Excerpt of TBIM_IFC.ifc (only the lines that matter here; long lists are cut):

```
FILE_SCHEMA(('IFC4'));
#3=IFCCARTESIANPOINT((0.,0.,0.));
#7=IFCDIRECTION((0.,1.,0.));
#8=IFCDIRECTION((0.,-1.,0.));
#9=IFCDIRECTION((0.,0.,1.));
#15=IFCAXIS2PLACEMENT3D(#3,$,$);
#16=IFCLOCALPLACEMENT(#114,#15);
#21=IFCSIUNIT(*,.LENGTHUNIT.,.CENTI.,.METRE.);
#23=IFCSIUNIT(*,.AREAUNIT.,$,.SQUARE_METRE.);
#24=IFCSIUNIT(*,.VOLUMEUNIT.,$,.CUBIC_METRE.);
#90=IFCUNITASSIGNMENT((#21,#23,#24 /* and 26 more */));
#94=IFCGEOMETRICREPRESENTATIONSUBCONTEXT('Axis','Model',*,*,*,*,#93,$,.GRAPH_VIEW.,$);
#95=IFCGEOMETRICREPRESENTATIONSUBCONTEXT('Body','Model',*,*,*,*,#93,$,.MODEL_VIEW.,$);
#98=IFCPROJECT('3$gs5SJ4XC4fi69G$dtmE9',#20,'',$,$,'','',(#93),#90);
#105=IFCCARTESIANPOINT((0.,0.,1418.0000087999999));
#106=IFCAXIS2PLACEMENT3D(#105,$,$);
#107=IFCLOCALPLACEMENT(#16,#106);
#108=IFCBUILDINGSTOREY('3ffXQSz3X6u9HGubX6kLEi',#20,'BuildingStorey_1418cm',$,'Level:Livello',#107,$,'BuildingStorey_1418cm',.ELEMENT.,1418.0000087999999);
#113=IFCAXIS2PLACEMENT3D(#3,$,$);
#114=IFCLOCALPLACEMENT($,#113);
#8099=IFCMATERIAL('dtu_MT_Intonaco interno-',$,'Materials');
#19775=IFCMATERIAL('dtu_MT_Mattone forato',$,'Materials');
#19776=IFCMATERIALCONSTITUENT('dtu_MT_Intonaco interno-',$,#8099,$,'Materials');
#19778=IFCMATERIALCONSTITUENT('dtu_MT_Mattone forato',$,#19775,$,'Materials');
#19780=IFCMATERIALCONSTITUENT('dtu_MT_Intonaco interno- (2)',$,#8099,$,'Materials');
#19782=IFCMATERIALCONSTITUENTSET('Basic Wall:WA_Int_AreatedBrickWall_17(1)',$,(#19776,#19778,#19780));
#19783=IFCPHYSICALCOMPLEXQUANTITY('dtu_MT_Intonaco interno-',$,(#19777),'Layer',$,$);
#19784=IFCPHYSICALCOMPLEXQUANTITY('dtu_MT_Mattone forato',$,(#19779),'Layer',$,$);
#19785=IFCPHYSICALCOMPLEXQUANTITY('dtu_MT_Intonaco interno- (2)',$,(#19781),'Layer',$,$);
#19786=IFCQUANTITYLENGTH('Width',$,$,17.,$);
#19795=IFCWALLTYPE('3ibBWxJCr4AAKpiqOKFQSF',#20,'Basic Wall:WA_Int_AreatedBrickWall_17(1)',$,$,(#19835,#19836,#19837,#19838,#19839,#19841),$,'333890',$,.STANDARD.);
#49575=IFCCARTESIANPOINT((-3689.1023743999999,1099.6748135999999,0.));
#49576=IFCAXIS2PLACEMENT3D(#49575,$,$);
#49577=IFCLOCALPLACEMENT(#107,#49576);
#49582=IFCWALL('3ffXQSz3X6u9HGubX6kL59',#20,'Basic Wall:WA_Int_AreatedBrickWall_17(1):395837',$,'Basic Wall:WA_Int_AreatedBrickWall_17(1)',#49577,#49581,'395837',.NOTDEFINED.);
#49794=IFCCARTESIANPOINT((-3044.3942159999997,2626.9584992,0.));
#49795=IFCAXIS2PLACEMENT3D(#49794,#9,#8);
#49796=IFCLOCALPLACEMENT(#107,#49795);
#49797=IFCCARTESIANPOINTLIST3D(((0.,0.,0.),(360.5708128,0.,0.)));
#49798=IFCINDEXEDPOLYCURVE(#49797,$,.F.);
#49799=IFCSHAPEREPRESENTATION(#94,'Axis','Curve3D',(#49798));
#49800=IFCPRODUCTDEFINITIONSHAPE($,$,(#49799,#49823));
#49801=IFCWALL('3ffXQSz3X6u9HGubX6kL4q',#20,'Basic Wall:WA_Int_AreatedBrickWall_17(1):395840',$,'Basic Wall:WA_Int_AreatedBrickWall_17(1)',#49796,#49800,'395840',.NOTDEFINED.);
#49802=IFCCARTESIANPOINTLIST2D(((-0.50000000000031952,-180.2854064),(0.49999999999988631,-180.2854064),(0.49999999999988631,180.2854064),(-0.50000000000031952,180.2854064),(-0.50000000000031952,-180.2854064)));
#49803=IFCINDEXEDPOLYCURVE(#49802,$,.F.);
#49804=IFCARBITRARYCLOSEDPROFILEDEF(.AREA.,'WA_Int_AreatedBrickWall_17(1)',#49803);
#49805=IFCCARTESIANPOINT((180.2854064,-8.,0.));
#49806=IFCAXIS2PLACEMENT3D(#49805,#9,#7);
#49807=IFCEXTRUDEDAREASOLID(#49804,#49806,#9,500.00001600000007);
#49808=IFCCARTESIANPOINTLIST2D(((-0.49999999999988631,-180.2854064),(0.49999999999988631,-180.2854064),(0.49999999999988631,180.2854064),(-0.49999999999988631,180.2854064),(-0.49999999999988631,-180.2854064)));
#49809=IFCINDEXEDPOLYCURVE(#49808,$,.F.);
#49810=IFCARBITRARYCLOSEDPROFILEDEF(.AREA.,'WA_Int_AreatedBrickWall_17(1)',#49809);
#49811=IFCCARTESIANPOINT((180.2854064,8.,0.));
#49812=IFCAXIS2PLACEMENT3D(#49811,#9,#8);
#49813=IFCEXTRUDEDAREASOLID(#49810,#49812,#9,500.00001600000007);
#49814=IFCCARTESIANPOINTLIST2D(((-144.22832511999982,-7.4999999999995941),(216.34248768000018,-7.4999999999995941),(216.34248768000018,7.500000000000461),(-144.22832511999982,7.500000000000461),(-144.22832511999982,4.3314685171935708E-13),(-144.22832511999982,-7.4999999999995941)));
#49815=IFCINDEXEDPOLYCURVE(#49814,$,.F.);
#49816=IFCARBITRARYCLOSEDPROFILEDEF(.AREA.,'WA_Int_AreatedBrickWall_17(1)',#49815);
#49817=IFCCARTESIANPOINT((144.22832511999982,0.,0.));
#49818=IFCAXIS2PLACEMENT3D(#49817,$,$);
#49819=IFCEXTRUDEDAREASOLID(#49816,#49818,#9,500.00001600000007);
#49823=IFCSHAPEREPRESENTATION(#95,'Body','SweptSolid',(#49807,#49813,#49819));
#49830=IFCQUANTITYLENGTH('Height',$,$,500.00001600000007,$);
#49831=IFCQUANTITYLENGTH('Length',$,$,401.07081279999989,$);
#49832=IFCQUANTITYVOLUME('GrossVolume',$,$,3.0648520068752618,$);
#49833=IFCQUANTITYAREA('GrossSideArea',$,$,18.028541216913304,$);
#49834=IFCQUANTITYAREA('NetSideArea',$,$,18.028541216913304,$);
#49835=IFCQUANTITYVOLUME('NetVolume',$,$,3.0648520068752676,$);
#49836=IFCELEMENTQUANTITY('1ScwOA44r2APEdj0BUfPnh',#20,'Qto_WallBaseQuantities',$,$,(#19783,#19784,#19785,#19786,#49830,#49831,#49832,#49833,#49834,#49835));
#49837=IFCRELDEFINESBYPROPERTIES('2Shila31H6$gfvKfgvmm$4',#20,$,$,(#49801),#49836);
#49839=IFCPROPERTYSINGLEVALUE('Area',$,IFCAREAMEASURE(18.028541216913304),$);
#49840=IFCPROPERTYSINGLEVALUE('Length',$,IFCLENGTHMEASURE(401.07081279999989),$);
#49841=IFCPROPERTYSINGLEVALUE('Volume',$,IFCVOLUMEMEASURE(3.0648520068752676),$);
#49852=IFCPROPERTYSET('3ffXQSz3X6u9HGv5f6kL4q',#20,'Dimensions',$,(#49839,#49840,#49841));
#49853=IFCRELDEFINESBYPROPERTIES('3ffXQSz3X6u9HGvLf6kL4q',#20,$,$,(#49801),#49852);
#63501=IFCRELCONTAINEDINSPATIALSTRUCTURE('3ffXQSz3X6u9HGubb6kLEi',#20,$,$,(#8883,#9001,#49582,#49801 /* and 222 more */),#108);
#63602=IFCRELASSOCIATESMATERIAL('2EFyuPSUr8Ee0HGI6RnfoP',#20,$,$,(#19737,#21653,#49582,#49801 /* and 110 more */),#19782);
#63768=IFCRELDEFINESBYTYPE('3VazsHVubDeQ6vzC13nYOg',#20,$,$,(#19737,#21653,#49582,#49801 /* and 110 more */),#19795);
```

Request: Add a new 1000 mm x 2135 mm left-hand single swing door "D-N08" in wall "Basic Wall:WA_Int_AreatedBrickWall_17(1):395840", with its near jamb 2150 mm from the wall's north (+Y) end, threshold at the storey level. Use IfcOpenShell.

```python
import numpy as np
import ifcopenshell
import ifcopenshell.api.feature
import ifcopenshell.api.geometry
import ifcopenshell.api.pset
import ifcopenshell.api.root
import ifcopenshell.api.spatial
import ifcopenshell.geom
import ifcopenshell.util.element
import ifcopenshell.util.placement
import ifcopenshell.util.representation
import ifcopenshell.util.shape
import ifcopenshell.util.unit

model = ifcopenshell.open("TBIM_IFC.ifc")
unit_scale = ifcopenshell.util.unit.calculate_unit_scale(model)
area_scale = ifcopenshell.util.unit.calculate_unit_scale(model, "AREAUNIT")
volume_scale = ifcopenshell.util.unit.calculate_unit_scale(model, "VOLUMEUNIT")
settings = ifcopenshell.geom.settings()


def volume(element):
    """Net volume in cubic metres, openings subtracted."""
    shape = ifcopenshell.geom.create_shape(settings, element)
    return ifcopenshell.util.shape.get_volume(shape.geometry)


wall = model.by_guid("3ffXQSz3X6u9HGubX6kL4q")
storey = ifcopenshell.util.element.get_container(wall, ifc_class="IfcBuildingStorey")
context = ifcopenshell.util.representation.get_context(model, "Model", "Body", "MODEL_VIEW")
before = volume(wall)

width, height, from_end, sill = 1, 2.135, 2.15, 0.0  # metres

# The wall runs along its own X axis, and the end named is its -X end.
wall_shape = ifcopenshell.geom.create_shape(settings, wall)
x, y, z = ifcopenshell.util.shape.get_vertices(wall_shape.geometry).T
start = x.min() + from_end
face, thickness = float(y.min()), float(y.max() - y.min())
wall_matrix = ifcopenshell.util.placement.get_local_placement(wall.ObjectPlacement)
level = ifcopenshell.util.placement.get_local_placement(storey.ObjectPlacement)[2, 3]


def in_wall(x, y):
    """Placement at x, y metres in the wall's axes, at sill height."""
    matrix = wall_matrix.copy()
    matrix[:, 3] = wall_matrix @ np.array([x / unit_scale, y / unit_scale, 0.0, 1.0])
    matrix[2, 3] = level + sill / unit_scale
    return matrix


# Opening: a box that overshoots both wall faces by 50 mm.
opening = ifcopenshell.api.root.create_entity(model, ifc_class="IfcOpeningElement", predefined_type="OPENING")
box = ifcopenshell.api.geometry.add_wall_representation(
    model, context=context, length=width, height=height, thickness=thickness + 0.1
)
ifcopenshell.api.geometry.assign_representation(model, product=opening, representation=box)
ifcopenshell.api.geometry.edit_object_placement(model, product=opening, matrix=in_wall(start, face - 0.05), is_si=False)
ifcopenshell.api.feature.add_feature(model, feature=opening, element=wall)

door = ifcopenshell.api.root.create_entity(model, ifc_class="IfcDoor", name="D-N08", predefined_type="DOOR")
door.OverallWidth, door.OverallHeight = width / unit_scale, height / unit_scale
door.OperationType = "SINGLE_SWING_LEFT"
body = ifcopenshell.api.geometry.add_door_representation(
    model,
    context=context,
    overall_width=door.OverallWidth,
    overall_height=door.OverallHeight,
    operation_type="SINGLE_SWING_LEFT",
    lining_properties={"LiningDepth": thickness / unit_scale, "ThresholdDepth": thickness / unit_scale},
)
ifcopenshell.api.geometry.assign_representation(model, product=door, representation=body)
ifcopenshell.api.spatial.assign_container(model, products=[door], relating_structure=storey)
ifcopenshell.api.feature.add_filling(model, opening=opening, element=door)

# The lining spans the wall, so the door starts at the wall face.
ifcopenshell.api.geometry.edit_object_placement(model, product=door, matrix=in_wall(start, face), is_si=False)

after = volume(wall)

# Update the wall's stored quantities.
qto = model.by_id(ifcopenshell.util.element.get_pset(wall, "Qto_WallBaseQuantities", should_inherit=False)["id"])
ifcopenshell.api.pset.edit_qto(model, qto=qto, properties={
    "NetSideArea": after / thickness / area_scale,
    "NetVolume": after / volume_scale,
})
pset = model.by_id(ifcopenshell.util.element.get_pset(wall, "Dimensions", should_inherit=False)["id"])
ifcopenshell.api.pset.edit_pset(model, pset=pset, properties={
    "Area": model.create_entity("IfcAreaMeasure", after / thickness / area_scale),
    "Volume": model.create_entity("IfcVolumeMeasure", after / volume_scale),
})

print(f"wall volume {before:.3f} -> {after:.3f} m3")

model.write("TBIM_IFC_rev.ifc")
```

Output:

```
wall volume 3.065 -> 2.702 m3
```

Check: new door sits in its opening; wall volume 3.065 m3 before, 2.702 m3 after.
